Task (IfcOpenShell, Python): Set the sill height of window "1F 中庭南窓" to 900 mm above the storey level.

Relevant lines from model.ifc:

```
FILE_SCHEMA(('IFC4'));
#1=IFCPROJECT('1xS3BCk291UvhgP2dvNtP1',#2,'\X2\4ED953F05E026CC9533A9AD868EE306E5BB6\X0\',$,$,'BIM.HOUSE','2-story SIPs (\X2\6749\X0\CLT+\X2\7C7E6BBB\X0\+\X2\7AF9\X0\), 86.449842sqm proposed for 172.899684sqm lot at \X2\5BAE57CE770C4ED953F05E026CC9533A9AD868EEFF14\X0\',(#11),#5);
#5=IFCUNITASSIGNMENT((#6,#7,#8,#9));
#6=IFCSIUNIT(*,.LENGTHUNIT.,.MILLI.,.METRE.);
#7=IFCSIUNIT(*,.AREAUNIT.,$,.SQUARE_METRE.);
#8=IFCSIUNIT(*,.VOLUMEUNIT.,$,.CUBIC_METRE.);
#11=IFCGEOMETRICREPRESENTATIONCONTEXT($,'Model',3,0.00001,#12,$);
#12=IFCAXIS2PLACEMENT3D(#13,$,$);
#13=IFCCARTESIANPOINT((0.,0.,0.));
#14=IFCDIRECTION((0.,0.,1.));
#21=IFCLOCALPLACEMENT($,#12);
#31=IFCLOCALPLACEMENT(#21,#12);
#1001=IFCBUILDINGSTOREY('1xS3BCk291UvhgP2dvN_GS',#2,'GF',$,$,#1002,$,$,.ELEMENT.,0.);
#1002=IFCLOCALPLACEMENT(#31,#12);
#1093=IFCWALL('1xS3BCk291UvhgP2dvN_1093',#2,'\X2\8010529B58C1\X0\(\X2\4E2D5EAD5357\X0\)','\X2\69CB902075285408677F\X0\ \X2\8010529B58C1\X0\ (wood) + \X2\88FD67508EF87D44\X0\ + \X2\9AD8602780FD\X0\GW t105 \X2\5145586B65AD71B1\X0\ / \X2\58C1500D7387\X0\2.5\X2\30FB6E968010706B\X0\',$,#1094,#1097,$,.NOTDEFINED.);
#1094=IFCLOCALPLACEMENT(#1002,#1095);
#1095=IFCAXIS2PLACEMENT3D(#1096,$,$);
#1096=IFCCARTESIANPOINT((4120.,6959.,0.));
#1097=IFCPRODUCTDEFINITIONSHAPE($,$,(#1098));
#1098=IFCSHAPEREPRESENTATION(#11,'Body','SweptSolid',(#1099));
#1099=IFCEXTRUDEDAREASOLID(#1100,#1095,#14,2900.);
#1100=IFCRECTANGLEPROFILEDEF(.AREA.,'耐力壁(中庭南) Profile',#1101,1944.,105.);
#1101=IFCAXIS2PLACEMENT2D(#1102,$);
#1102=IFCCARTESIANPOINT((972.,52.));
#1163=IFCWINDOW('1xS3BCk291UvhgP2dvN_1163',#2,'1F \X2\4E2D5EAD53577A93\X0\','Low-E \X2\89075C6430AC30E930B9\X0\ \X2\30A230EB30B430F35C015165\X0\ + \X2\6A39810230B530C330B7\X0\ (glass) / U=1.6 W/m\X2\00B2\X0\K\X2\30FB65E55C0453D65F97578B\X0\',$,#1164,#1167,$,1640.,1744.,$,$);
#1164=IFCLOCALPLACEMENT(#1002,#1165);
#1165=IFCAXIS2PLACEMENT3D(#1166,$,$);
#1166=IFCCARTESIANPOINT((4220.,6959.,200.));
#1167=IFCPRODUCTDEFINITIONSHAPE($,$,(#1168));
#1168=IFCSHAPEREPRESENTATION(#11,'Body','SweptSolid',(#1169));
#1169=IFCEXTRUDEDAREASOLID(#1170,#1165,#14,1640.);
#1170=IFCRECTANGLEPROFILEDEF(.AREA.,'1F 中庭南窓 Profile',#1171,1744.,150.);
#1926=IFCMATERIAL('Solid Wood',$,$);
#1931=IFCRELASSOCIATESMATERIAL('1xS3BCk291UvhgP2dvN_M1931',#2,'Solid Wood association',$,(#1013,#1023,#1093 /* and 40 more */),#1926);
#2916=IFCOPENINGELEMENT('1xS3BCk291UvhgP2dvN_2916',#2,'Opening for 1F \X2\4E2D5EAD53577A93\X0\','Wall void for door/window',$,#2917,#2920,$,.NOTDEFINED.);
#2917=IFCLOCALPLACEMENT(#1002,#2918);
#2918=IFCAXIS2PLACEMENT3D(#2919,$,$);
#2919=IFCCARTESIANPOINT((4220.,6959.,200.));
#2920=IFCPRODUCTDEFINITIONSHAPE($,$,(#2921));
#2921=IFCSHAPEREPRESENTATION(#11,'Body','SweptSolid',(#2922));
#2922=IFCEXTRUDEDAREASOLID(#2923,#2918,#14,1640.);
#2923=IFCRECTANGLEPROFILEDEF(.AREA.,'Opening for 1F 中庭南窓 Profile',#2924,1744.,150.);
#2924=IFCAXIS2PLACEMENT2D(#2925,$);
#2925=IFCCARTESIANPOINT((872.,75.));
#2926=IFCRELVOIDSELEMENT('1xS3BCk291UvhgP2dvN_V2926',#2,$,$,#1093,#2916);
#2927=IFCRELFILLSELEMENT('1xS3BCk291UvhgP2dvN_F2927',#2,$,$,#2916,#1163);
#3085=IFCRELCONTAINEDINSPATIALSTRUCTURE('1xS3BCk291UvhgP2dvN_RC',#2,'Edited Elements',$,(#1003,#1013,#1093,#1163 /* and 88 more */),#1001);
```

```python
import numpy as np
import ifcopenshell
import ifcopenshell.api.geometry
import ifcopenshell.geom
import ifcopenshell.util.element
import ifcopenshell.util.placement
import ifcopenshell.util.shape
import ifcopenshell.util.unit

model = ifcopenshell.open("model.ifc")
unit_scale = ifcopenshell.util.unit.calculate_unit_scale(model)

window = model.by_guid("1xS3BCk291UvhgP2dvN_1163")
opening = window.FillsVoids[0].RelatingOpeningElement
storey = ifcopenshell.util.element.get_container(window, ifc_class="IfcBuildingStorey")
level = ifcopenshell.util.placement.get_local_placement(storey.ObjectPlacement)[2, 3]

# The opening's origin need not be at the sill, so measure its lowest point.
shape = ifcopenshell.geom.create_shape(ifcopenshell.geom.settings(), opening)
bottom = ifcopenshell.util.shape.get_shape_bottom_elevation(shape, shape.geometry) / unit_scale
dz = level + 0.9 / unit_scale - bottom

shift = np.array([0.0, 0.0, dz])
# The window is not placed relative to its opening, so move both.
for product in (opening, window):
    matrix = ifcopenshell.util.placement.get_local_placement(product.ObjectPlacement)
    matrix[:3, 3] += shift
    ifcopenshell.api.geometry.edit_object_placement(model, product=product, matrix=matrix, is_si=False)

print(f"moved by {dz * unit_scale:+.3f} m")

model.write("model_rev.ifc")
```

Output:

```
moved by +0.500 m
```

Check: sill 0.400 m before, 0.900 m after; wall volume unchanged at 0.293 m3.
